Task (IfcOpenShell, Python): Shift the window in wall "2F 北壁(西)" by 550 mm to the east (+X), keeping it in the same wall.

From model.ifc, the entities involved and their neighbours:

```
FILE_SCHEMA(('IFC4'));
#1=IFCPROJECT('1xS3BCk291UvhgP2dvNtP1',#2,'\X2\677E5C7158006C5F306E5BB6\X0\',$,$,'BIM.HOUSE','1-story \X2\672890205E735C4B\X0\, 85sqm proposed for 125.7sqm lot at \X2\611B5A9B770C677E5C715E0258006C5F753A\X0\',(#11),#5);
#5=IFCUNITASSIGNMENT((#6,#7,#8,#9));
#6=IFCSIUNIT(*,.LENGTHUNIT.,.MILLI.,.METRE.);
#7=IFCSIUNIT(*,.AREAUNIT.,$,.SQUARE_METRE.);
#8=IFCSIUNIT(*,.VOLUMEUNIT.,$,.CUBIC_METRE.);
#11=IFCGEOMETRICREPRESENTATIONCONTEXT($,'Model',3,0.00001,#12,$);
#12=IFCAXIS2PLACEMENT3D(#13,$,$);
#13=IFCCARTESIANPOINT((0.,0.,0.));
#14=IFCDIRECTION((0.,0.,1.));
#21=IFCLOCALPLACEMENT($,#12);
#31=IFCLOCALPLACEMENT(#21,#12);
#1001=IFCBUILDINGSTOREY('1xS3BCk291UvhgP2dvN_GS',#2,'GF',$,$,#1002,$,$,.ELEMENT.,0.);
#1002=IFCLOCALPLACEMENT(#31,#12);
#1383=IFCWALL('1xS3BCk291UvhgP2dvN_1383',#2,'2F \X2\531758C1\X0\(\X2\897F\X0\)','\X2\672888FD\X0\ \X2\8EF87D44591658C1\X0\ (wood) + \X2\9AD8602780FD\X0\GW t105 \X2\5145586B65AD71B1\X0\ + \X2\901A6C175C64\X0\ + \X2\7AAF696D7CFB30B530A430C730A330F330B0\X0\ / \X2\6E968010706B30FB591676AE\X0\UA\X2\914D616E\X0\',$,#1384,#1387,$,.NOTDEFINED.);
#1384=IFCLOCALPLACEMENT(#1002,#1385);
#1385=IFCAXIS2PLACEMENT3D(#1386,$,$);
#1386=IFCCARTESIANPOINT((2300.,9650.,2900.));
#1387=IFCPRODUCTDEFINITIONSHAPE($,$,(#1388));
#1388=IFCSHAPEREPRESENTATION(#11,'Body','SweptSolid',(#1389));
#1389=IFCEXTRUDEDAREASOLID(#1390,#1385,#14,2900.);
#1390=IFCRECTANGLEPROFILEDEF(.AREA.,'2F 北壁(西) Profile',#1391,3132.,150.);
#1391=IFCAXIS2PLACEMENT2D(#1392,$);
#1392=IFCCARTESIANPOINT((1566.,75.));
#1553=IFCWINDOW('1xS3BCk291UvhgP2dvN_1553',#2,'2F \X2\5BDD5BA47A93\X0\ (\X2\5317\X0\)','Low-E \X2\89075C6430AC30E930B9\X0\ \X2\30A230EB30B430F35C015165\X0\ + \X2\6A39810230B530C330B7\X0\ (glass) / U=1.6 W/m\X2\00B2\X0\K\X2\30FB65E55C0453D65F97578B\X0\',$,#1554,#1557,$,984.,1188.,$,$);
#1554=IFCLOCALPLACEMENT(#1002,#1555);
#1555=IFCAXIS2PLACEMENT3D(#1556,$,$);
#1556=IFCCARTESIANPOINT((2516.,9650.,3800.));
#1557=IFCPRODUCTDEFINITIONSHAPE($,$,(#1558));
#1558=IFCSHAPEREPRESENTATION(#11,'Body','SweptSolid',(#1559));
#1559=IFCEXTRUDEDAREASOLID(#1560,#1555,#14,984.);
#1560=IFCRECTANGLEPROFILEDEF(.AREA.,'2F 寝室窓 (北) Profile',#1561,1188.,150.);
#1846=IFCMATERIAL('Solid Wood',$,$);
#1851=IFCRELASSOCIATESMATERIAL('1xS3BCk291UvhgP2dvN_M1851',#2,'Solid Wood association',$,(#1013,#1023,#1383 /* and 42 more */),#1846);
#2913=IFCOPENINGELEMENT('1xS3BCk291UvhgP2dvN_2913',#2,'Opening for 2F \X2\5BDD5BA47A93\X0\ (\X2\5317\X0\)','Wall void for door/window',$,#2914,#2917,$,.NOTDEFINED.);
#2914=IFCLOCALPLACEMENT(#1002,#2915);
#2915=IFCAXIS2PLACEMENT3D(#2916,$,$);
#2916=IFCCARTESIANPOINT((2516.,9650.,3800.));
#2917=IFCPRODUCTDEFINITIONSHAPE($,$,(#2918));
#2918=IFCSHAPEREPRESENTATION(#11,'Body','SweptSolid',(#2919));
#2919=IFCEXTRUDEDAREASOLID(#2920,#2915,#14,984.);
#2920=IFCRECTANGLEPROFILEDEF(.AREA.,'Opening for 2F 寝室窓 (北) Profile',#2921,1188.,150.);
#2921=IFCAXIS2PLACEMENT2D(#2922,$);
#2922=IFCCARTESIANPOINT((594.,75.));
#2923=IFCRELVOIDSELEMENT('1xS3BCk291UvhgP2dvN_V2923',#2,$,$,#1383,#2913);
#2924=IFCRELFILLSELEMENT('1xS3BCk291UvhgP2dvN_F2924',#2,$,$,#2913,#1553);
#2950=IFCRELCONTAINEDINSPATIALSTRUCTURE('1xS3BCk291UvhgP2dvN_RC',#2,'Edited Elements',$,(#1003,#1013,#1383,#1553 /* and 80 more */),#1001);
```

```python
import ifcopenshell
import ifcopenshell.api.geometry
import ifcopenshell.util.placement
import ifcopenshell.util.unit

model = ifcopenshell.open("model.ifc")
unit_scale = ifcopenshell.util.unit.calculate_unit_scale(model)

window = model.by_guid("1xS3BCk291UvhgP2dvN_1553")
opening = window.FillsVoids[0].RelatingOpeningElement
wall = opening.VoidsElements[0].RelatingBuildingElement

wall_matrix = ifcopenshell.util.placement.get_local_placement(wall.ObjectPlacement)
shift = wall_matrix[:3, 0] * 0.55 / unit_scale
before = ifcopenshell.util.placement.get_local_placement(window.ObjectPlacement)[:3, 3].copy()

# The window is not placed relative to its opening, so move both.
for product in (opening, window):
    matrix = ifcopenshell.util.placement.get_local_placement(product.ObjectPlacement)
    matrix[:3, 3] += shift
    ifcopenshell.api.geometry.edit_object_placement(model, product=product, matrix=matrix, is_si=False)

after = ifcopenshell.util.placement.get_local_placement(window.ObjectPlacement)[:3, 3]
print("window moved by", (after - before).round(3) + 0.0)

model.write("model_rev.ifc")
```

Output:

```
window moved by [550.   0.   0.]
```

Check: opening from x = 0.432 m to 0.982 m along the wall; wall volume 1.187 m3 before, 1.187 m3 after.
